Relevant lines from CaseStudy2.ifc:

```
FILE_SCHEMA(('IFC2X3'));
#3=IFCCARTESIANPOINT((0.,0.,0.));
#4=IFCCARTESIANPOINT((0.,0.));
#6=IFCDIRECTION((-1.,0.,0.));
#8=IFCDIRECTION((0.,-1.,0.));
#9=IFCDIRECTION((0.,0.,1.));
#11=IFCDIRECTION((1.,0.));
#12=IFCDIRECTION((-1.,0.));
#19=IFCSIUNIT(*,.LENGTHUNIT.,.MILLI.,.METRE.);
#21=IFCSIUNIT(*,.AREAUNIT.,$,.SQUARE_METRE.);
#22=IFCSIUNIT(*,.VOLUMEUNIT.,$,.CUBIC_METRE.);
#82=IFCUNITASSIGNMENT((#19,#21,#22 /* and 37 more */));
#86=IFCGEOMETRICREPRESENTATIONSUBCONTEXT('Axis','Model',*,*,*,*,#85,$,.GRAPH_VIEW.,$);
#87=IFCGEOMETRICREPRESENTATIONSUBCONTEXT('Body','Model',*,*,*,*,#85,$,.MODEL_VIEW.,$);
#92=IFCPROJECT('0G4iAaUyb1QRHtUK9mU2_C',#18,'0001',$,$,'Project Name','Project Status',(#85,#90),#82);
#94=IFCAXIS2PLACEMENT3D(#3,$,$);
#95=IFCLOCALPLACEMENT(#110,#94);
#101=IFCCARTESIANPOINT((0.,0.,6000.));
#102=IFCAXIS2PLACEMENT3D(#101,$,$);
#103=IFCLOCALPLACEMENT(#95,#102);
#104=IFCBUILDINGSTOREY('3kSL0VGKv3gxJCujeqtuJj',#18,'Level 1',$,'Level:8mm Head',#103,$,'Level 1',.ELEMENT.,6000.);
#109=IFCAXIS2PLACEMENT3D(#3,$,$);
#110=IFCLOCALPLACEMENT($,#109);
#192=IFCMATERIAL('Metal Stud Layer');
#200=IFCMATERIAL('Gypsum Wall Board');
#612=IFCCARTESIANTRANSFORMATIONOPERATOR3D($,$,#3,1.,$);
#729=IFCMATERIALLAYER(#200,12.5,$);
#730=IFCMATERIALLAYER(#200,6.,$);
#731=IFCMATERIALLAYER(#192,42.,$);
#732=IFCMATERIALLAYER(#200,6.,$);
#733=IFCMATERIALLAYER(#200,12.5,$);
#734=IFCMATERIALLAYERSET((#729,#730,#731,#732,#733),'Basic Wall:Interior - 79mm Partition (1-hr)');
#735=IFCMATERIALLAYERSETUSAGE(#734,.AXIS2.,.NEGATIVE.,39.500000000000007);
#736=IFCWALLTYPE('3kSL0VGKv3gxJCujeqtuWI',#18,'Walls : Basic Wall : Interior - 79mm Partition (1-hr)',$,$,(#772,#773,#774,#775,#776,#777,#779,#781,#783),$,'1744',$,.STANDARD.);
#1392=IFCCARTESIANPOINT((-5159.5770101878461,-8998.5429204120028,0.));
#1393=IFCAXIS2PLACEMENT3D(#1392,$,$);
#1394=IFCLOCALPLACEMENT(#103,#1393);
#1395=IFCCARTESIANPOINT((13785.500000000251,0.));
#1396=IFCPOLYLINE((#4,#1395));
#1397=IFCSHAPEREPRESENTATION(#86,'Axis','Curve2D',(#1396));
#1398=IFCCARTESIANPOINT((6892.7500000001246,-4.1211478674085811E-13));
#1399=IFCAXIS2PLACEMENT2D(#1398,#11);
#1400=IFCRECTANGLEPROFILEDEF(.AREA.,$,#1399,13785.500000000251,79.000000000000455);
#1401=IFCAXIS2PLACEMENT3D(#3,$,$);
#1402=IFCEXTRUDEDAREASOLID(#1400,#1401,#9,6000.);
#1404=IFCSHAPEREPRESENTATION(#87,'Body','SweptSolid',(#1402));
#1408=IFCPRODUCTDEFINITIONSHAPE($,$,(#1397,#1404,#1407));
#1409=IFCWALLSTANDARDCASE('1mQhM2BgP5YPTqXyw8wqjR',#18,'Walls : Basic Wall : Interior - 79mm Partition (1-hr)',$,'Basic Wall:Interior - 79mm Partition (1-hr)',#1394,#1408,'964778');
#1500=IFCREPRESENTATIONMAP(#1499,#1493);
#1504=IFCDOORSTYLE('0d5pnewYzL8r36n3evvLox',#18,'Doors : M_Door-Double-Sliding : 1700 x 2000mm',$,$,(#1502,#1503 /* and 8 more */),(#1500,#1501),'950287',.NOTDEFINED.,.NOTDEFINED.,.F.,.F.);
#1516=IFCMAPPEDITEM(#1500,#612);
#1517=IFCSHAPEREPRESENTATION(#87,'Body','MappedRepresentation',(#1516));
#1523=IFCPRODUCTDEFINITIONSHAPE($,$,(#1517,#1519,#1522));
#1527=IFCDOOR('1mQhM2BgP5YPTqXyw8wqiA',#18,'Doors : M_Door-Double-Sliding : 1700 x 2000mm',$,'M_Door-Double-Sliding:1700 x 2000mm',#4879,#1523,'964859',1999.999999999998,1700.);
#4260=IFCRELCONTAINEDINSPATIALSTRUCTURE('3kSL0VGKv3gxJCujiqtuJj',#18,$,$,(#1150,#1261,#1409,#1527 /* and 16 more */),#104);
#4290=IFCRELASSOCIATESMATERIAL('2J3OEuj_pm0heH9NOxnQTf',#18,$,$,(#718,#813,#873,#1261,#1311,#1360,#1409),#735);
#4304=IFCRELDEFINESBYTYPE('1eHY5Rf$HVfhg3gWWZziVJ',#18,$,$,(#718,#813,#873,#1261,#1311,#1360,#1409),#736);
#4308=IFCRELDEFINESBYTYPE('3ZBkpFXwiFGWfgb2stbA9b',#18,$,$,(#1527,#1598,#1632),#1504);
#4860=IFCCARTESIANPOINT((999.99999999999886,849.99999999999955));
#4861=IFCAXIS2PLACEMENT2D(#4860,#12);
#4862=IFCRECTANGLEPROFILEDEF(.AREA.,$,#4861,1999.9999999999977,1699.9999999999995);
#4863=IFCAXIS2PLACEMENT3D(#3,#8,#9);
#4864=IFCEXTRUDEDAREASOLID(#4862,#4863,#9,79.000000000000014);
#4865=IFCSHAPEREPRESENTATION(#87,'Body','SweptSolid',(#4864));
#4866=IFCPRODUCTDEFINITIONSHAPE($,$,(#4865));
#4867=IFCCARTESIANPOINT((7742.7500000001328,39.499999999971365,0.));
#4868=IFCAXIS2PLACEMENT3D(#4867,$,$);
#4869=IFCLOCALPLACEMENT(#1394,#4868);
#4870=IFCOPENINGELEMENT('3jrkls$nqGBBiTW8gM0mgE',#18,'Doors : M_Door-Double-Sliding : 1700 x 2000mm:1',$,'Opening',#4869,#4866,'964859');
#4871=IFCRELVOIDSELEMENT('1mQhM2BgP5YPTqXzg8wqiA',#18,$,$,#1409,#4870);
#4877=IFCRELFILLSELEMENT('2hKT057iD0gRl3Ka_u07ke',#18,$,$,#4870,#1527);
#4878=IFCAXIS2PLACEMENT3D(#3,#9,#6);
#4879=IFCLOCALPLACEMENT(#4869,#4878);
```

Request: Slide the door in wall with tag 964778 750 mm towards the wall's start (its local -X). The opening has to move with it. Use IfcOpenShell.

```python
import ifcopenshell
import ifcopenshell.api.geometry
import ifcopenshell.util.placement
import ifcopenshell.util.unit

model = ifcopenshell.open("CaseStudy2.ifc")
unit_scale = ifcopenshell.util.unit.calculate_unit_scale(model)

door = model.by_guid("1mQhM2BgP5YPTqXyw8wqiA")
opening = door.FillsVoids[0].RelatingOpeningElement
wall = opening.VoidsElements[0].RelatingBuildingElement

wall_matrix = ifcopenshell.util.placement.get_local_placement(wall.ObjectPlacement)
shift = wall_matrix[:3, 0] * -0.75 / unit_scale
before = ifcopenshell.util.placement.get_local_placement(door.ObjectPlacement)[:3, 3].copy()

# The door is placed relative to its opening, so it follows when the opening moves.
matrix = ifcopenshell.util.placement.get_local_placement(opening.ObjectPlacement)
matrix[:3, 3] += shift
ifcopenshell.api.geometry.edit_object_placement(
    model, product=opening, matrix=matrix, is_si=False, should_transform_children=True
)

after = ifcopenshell.util.placement.get_local_placement(door.ObjectPlacement)[:3, 3]
print("door moved by", (after - before).round(3) + 0.0)

model.write("CaseStudy2_rev.ifc")
```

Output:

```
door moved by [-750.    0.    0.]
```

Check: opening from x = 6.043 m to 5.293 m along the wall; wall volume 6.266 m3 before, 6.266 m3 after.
